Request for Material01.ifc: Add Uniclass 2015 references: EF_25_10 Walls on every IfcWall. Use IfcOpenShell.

First a look at what the model holds.

```python
import ifcopenshell

model = ifcopenshell.open("Material01.ifc")
print(model.schema)
print("classifications:", [c.Name for c in model.by_type("IfcClassification")])
for ifc_class in ("IfcDoor", "IfcRoof", "IfcStair", "IfcWall", "IfcWindow"):
    print(ifc_class, len(model.by_type(ifc_class)))
```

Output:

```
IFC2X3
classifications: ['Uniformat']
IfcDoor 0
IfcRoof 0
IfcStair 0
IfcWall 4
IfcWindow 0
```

```python
import ifcopenshell
import ifcopenshell.api.classification

model = ifcopenshell.open("Material01.ifc")

# IFC2X3 requires Source and Edition and has no link from the project to the system.
system = model.create_entity("IfcClassification", Source="NBS", Edition="2015", Name="Uniclass 2015")

codes = {
    "IfcWall": ("EF_25_10", "Walls"),
}
for ifc_class, (code, name) in codes.items():
    products = model.by_type(ifc_class)
    ifcopenshell.api.classification.add_reference(
        model, products=products, classification=system, identification=code, name=name
    )
    print(code, len(products))

model.write("Material01_edited.ifc")
```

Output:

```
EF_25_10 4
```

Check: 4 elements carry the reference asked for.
